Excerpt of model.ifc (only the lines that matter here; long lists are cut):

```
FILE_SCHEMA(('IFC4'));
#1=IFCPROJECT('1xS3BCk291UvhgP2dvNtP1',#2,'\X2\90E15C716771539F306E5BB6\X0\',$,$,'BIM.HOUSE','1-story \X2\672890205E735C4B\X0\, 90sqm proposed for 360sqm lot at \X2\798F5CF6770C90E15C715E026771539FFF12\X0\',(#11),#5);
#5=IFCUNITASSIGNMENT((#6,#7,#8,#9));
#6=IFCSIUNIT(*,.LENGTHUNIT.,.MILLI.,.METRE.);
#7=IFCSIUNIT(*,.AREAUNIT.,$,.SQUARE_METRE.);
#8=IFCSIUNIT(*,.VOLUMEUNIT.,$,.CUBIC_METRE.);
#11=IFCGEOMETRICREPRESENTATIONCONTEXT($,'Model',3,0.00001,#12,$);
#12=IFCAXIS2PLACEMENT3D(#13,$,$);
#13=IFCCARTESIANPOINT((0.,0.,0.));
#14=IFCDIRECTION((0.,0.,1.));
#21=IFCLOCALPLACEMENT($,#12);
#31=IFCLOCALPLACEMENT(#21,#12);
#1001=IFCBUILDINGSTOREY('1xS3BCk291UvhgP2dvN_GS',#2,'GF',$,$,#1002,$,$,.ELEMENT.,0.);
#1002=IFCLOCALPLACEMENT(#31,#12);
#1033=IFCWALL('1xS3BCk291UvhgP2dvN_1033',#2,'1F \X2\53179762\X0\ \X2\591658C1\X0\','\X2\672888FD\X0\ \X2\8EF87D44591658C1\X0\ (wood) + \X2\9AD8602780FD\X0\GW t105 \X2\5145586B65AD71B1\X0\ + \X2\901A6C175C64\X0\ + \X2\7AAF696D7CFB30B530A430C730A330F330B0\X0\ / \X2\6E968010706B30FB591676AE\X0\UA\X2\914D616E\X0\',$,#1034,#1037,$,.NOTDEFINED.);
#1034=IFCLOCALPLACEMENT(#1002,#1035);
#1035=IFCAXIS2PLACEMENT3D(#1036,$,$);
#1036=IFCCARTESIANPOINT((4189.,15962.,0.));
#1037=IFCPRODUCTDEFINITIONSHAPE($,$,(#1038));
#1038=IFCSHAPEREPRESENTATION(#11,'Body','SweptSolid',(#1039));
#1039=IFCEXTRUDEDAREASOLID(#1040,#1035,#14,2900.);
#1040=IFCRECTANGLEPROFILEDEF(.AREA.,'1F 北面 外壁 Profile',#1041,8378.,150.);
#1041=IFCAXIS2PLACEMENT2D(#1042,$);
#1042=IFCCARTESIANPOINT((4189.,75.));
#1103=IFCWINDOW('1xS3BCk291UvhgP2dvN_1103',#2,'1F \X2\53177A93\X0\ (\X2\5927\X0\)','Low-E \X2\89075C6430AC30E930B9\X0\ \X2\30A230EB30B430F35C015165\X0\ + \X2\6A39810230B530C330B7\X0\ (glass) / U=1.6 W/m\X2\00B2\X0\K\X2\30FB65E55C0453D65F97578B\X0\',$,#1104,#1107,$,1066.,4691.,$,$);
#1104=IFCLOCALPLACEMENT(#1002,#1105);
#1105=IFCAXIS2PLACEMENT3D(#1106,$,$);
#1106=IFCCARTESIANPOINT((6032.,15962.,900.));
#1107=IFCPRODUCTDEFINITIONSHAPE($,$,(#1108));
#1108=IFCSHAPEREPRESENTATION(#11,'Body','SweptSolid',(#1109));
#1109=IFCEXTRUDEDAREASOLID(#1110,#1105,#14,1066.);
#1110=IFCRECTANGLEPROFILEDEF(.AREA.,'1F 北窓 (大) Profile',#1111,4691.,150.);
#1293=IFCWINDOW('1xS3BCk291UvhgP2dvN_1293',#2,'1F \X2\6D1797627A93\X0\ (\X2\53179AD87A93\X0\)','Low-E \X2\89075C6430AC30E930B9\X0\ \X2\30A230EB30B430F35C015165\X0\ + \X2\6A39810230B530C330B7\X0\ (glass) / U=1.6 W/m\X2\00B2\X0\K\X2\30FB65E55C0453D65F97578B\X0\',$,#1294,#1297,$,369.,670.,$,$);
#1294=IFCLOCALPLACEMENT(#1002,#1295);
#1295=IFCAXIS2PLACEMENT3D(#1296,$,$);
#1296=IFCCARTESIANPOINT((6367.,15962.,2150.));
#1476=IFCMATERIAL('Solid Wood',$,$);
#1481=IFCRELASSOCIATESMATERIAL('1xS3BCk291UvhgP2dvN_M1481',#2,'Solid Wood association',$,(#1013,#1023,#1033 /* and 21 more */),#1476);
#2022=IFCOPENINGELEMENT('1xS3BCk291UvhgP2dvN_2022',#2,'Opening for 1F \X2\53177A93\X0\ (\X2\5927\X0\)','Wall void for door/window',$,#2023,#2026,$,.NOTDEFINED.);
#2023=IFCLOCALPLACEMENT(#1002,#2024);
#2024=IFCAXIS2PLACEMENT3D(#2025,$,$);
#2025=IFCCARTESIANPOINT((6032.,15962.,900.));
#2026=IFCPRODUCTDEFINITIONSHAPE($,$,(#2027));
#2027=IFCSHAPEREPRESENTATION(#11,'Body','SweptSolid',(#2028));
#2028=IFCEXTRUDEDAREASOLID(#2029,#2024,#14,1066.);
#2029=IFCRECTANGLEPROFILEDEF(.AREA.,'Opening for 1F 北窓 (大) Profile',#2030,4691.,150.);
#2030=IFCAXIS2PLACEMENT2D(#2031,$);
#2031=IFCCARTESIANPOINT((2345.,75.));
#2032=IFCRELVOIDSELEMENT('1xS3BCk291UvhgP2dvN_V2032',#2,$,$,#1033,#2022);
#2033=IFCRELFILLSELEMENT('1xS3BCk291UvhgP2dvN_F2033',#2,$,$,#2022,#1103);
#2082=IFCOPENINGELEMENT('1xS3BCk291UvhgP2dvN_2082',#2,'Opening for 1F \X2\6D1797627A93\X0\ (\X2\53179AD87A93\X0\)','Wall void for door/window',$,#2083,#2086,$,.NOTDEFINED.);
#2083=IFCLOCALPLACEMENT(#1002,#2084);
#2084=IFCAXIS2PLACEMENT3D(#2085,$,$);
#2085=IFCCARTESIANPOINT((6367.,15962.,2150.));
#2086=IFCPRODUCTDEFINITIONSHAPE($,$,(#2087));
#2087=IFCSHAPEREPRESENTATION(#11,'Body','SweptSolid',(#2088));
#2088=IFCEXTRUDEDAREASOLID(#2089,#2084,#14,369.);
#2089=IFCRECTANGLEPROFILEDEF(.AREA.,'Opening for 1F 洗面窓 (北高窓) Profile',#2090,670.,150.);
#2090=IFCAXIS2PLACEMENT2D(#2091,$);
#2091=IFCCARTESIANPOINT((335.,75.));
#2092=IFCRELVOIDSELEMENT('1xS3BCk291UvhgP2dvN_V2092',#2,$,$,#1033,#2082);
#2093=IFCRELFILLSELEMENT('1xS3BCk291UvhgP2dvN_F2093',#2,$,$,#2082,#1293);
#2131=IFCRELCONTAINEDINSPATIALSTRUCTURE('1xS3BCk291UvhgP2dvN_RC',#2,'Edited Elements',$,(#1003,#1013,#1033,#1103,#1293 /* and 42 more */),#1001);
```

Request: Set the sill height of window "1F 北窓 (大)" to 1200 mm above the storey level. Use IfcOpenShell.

```python
import numpy as np
import ifcopenshell
import ifcopenshell.api.geometry
import ifcopenshell.geom
import ifcopenshell.util.element
import ifcopenshell.util.placement
import ifcopenshell.util.shape
import ifcopenshell.util.unit

model = ifcopenshell.open("model.ifc")
unit_scale = ifcopenshell.util.unit.calculate_unit_scale(model)

window = model.by_guid("1xS3BCk291UvhgP2dvN_1103")
opening = window.FillsVoids[0].RelatingOpeningElement
storey = ifcopenshell.util.element.get_container(window, ifc_class="IfcBuildingStorey")
level = ifcopenshell.util.placement.get_local_placement(storey.ObjectPlacement)[2, 3]

# The opening's origin need not be at the sill, so measure its lowest point.
shape = ifcopenshell.geom.create_shape(ifcopenshell.geom.settings(), opening)
bottom = ifcopenshell.util.shape.get_shape_bottom_elevation(shape, shape.geometry) / unit_scale
dz = level + 1.2 / unit_scale - bottom

shift = np.array([0.0, 0.0, dz])
# The window is not placed relative to its opening, so move both.
for product in (opening, window):
    matrix = ifcopenshell.util.placement.get_local_placement(product.ObjectPlacement)
    matrix[:3, 3] += shift
    ifcopenshell.api.geometry.edit_object_placement(model, product=product, matrix=matrix, is_si=False)

print(f"moved by {dz * unit_scale:+.3f} m")

model.write("model_edited.ifc")
```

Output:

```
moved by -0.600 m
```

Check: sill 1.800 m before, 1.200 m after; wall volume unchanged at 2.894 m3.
